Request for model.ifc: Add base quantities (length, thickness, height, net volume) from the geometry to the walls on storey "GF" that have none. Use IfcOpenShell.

First a look at what the model holds.

```python
import ifcopenshell
import ifcopenshell.util.element
import ifcopenshell.util.unit

model = ifcopenshell.open("model.ifc")
print(model.schema)
for unit_type in ("LENGTHUNIT", "AREAUNIT", "VOLUMEUNIT"):
    print(unit_type, ifcopenshell.util.unit.calculate_unit_scale(model, unit_type))
storey = next(s for s in model.by_type("IfcBuildingStorey") if s.Name == "GF")
walls = [e for e in ifcopenshell.util.element.get_decomposition(storey) if e.is_a("IfcWall")]
for e in sorted(walls, key=lambda e: e.id()):
    print(e.id(), e.is_a(), e.Name, list(ifcopenshell.util.element.get_psets(e, qtos_only=True)), sep=" | ")
```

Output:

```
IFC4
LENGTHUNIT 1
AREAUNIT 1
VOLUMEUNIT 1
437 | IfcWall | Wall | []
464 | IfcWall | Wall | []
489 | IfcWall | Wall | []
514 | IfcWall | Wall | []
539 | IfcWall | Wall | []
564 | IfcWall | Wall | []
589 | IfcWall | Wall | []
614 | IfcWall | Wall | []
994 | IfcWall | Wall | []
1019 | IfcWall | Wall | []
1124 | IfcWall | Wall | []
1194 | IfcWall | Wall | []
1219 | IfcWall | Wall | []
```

```python
import ifcopenshell
import ifcopenshell.api.pset
import ifcopenshell.geom
import ifcopenshell.util.element
import ifcopenshell.util.shape
import ifcopenshell.util.unit

model = ifcopenshell.open("model.ifc")
unit_scale = ifcopenshell.util.unit.calculate_unit_scale(model)
volume_scale = ifcopenshell.util.unit.calculate_unit_scale(model, "VOLUMEUNIT")
settings = ifcopenshell.geom.settings()

storey = next(s for s in model.by_type("IfcBuildingStorey") if s.Name == "GF")
walls = [e for e in ifcopenshell.util.element.get_decomposition(storey) if e.is_a("IfcWall")]

for e in sorted(walls, key=lambda e: e.id()):
    if ifcopenshell.util.element.get_psets(e, qtos_only=True, should_inherit=False):
        continue
    # Geometry comes back in metres, in the element's own axes.
    shape = ifcopenshell.geom.create_shape(settings, e)
    values = {
        "Length": ifcopenshell.util.shape.get_x(shape.geometry) / unit_scale,
        "Width": ifcopenshell.util.shape.get_y(shape.geometry) / unit_scale,
        "Height": ifcopenshell.util.shape.get_z(shape.geometry) / unit_scale,
        "NetVolume": ifcopenshell.util.shape.get_volume(shape.geometry) / volume_scale,
    }
    qto = ifcopenshell.api.pset.add_qto(model, product=e, name="Qto_WallBaseQuantities")
    ifcopenshell.api.pset.edit_qto(model, qto=qto, properties=values)
    print(e.id(), {k: round(v, 3) for k, v in values.items()})

model.write("model-out.ifc")
```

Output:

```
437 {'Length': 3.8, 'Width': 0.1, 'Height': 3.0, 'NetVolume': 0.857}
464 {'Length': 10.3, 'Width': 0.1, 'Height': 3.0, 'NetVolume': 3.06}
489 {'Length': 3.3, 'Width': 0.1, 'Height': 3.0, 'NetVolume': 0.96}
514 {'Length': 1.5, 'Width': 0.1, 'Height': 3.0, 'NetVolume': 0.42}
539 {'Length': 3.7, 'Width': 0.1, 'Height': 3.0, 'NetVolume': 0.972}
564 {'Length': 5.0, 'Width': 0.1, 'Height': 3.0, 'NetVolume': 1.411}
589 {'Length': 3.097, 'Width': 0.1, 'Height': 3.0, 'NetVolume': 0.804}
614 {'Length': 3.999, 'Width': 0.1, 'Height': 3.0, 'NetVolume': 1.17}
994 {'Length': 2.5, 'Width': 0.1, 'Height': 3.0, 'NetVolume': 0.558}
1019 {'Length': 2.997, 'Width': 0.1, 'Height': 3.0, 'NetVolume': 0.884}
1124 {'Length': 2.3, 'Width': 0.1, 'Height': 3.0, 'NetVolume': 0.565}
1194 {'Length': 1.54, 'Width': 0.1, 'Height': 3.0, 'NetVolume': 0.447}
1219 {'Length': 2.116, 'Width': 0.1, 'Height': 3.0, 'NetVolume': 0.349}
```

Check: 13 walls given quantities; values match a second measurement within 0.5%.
